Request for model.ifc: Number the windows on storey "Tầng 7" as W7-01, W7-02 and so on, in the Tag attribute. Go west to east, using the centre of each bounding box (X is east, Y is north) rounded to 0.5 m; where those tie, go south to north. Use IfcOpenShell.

First a look at what the model holds.

```python
import ifcopenshell
import ifcopenshell.util.element
import ifcopenshell.util.placement

model = ifcopenshell.open("model.ifc")
print(model.schema)
storey = next(s for s in model.by_type("IfcBuildingStorey") if s.Name == "Tầng 7")
windows = [e for e in ifcopenshell.util.element.get_decomposition(storey) if e.is_a("IfcWindow")]
for e in sorted(windows, key=lambda e: e.id()):
    origin = ifcopenshell.util.placement.get_local_placement(e.ObjectPlacement)[:3, 3]
    print(e.id(), e.Tag, e.Name, origin.round(2) + 0.0, sep=" | ")
```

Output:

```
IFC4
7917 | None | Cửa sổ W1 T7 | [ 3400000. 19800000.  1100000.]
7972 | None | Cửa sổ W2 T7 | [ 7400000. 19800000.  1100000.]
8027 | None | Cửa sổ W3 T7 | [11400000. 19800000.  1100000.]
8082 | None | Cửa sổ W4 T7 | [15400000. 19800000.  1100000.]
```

```python
import ifcopenshell
import ifcopenshell.geom
import ifcopenshell.util.element
import ifcopenshell.util.shape

model = ifcopenshell.open("model.ifc")
settings = ifcopenshell.geom.settings()
settings.set("use-world-coords", True)


def centre(element):
    shape = ifcopenshell.geom.create_shape(settings, element)
    return ifcopenshell.util.shape.get_bbox_centroid(shape.geometry)


storey = next(s for s in model.by_type("IfcBuildingStorey") if s.Name == "Tầng 7")
windows = [e for e in ifcopenshell.util.element.get_decomposition(storey) if e.is_a("IfcWindow")]

# Insertion points can sit at a corner or the storey origin, so sort by the geometry (in metres).
centres = {e: centre(e) for e in windows}
windows.sort(key=lambda e: (round(centres[e][0] / 0.5), centres[e][1]))

for i, e in enumerate(windows, start=1):
    number = f"W7-{i:02d}"
    e.Tag = number
    print(e.id(), number)

model.write("model-out.ifc")
```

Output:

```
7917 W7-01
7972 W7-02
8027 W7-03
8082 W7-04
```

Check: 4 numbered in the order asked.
